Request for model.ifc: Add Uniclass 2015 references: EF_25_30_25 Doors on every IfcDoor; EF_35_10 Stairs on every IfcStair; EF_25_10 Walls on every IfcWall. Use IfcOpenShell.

First a look at what the model holds.

```python
import ifcopenshell

model = ifcopenshell.open("model.ifc")
print(model.schema)
print("classifications:", [c.Name for c in model.by_type("IfcClassification")])
for ifc_class in ("IfcDoor", "IfcRoof", "IfcStair", "IfcWall", "IfcWindow"):
    print(ifc_class, len(model.by_type(ifc_class)))
```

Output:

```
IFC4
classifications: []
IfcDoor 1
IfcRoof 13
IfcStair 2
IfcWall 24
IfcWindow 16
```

```python
import ifcopenshell
import ifcopenshell.api.classification

model = ifcopenshell.open("model.ifc")

system = ifcopenshell.api.classification.add_classification(model, classification="Uniclass 2015")

codes = {
    "IfcDoor": ("EF_25_30_25", "Doors"),
    "IfcStair": ("EF_35_10", "Stairs"),
    "IfcWall": ("EF_25_10", "Walls"),
}
for ifc_class, (code, name) in codes.items():
    products = model.by_type(ifc_class)
    ifcopenshell.api.classification.add_reference(
        model, products=products, classification=system, identification=code, name=name
    )
    print(code, len(products))

model.write("model_updated.ifc")
```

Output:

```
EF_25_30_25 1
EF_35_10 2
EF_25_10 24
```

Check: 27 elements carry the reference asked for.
